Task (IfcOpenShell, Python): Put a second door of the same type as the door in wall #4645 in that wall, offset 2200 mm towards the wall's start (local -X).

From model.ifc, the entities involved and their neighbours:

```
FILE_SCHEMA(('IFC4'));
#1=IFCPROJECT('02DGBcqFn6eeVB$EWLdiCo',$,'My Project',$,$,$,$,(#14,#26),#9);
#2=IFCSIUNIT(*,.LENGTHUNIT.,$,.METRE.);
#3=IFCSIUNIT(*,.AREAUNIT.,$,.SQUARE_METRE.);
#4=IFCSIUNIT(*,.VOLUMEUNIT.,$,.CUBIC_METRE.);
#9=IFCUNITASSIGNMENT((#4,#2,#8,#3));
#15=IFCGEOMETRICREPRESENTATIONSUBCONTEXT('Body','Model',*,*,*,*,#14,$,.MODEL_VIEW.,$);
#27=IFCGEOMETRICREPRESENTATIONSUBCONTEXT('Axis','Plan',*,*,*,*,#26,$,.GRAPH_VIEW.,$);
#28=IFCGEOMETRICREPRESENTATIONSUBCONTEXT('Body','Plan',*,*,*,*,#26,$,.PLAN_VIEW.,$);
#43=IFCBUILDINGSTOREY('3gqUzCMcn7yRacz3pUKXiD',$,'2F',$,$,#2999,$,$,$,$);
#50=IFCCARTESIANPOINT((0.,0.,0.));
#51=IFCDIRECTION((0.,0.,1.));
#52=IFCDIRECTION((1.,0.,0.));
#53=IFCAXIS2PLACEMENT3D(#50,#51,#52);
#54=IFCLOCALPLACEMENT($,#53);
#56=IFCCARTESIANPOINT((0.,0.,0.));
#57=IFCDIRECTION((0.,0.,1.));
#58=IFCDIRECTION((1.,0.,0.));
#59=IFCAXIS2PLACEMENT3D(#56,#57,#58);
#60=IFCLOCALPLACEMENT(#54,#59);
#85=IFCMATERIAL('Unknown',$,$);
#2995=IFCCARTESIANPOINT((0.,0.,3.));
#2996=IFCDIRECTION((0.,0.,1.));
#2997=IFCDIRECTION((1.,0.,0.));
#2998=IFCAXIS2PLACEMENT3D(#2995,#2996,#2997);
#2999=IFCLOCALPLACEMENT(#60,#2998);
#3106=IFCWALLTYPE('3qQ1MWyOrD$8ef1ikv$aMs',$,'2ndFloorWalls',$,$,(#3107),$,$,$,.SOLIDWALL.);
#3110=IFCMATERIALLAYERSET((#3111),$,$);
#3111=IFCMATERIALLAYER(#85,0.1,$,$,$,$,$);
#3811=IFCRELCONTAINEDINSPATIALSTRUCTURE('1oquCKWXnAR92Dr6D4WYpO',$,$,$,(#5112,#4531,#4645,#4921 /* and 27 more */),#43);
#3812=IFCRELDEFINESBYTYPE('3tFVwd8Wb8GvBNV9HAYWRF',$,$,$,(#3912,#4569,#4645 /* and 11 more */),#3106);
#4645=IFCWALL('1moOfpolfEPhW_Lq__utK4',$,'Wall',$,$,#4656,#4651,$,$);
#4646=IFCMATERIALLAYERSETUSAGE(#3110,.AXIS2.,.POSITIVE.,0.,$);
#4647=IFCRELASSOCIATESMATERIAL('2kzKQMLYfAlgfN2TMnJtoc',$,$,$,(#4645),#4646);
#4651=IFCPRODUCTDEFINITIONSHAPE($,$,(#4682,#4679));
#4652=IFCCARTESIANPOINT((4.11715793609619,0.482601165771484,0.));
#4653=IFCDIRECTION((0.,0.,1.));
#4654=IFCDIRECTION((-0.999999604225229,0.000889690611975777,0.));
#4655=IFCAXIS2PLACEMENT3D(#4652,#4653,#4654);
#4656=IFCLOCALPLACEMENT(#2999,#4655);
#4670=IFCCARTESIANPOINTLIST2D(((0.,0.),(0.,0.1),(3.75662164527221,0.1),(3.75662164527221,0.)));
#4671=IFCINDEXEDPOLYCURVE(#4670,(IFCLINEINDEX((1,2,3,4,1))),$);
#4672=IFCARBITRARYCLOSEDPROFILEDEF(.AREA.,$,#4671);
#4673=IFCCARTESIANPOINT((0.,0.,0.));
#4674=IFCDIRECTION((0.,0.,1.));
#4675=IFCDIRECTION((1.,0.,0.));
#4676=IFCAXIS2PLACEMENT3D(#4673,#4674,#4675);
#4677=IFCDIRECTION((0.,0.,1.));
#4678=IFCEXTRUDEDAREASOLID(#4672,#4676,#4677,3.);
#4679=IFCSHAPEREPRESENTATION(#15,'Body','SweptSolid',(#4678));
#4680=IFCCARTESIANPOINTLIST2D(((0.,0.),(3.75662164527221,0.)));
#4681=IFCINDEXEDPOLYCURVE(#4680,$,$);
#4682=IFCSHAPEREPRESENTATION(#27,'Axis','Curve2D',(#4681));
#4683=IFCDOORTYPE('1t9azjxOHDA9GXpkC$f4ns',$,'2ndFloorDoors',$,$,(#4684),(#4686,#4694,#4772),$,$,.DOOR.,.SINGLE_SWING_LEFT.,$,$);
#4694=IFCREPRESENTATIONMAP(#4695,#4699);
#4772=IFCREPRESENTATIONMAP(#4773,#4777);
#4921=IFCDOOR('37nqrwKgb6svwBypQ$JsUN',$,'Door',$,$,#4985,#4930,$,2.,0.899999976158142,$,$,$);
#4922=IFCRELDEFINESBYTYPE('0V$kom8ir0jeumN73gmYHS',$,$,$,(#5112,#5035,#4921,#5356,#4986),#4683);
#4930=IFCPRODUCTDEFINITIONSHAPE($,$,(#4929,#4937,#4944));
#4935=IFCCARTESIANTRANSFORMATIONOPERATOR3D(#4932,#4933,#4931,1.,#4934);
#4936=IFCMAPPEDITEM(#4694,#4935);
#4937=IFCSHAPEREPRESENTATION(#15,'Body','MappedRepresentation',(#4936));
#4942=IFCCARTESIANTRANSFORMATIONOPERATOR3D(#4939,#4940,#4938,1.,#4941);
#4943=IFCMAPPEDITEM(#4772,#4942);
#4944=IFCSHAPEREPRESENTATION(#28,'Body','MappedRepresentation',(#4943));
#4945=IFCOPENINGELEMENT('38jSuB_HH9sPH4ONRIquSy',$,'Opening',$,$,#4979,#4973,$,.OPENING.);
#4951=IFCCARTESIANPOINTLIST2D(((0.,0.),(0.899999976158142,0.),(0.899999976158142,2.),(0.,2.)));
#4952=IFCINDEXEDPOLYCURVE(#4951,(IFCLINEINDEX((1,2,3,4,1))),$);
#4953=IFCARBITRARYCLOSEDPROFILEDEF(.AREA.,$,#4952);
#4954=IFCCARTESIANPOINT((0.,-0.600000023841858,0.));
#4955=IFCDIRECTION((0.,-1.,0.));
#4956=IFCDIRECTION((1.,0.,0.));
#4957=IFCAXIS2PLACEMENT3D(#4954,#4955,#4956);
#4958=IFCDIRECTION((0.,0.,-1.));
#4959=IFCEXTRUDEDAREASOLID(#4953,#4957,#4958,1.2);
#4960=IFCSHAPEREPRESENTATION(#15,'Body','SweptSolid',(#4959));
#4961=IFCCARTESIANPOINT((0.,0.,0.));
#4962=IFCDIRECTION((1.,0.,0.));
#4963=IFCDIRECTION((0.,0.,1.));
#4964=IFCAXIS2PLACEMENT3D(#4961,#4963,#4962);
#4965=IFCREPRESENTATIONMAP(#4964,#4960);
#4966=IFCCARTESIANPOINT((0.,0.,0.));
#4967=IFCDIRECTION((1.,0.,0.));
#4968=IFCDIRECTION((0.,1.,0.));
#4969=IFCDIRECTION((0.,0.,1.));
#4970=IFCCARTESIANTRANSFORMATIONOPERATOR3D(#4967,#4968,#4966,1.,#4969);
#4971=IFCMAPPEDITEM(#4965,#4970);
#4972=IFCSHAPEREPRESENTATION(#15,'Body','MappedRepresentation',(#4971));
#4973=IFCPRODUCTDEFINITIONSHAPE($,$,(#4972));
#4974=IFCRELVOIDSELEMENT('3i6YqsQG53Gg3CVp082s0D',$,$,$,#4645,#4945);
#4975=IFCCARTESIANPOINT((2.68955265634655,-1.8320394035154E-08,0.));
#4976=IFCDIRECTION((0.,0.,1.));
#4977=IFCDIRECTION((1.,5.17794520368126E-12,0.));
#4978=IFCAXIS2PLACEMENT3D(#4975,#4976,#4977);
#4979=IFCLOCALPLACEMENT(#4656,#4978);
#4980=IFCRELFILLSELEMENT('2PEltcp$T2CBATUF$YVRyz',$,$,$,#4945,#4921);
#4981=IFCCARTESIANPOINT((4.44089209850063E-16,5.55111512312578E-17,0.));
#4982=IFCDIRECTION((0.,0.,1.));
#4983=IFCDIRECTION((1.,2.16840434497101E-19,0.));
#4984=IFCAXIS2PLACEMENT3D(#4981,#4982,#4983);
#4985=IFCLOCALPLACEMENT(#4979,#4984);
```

```python
import ifcopenshell
import ifcopenshell.api.feature
import ifcopenshell.api.geometry
import ifcopenshell.api.root
import ifcopenshell.geom
import ifcopenshell.util.element
import ifcopenshell.util.placement
import ifcopenshell.util.shape
import ifcopenshell.util.unit

model = ifcopenshell.open("model.ifc")
unit_scale = ifcopenshell.util.unit.calculate_unit_scale(model)
settings = ifcopenshell.geom.settings()


def volume(element):
    """Net volume in cubic metres, openings subtracted."""
    shape = ifcopenshell.geom.create_shape(settings, element)
    return ifcopenshell.util.shape.get_volume(shape.geometry)


door = model.by_guid("37nqrwKgb6svwBypQ$JsUN")
opening = door.FillsVoids[0].RelatingOpeningElement
wall = opening.VoidsElements[0].RelatingBuildingElement
before = volume(wall)
shift = ifcopenshell.util.placement.get_local_placement(wall.ObjectPlacement)[:3, 0] * -2.2 / unit_scale

# copy_class copies the void relationship, type, container and properties, but no geometry.
new_opening = ifcopenshell.api.root.copy_class(model, product=opening)
new_opening.Representation = ifcopenshell.util.element.copy_deep(
    model, opening.Representation, exclude=["IfcGeometricRepresentationContext", "IfcRepresentationMap"]
)
new_door = ifcopenshell.api.root.copy_class(model, product=door)
new_door.Representation = ifcopenshell.util.element.copy_deep(
    model, door.Representation, exclude=["IfcGeometricRepresentationContext", "IfcRepresentationMap"]
)
ifcopenshell.api.feature.add_filling(model, opening=new_opening, element=new_door)

for old, new in ((opening, new_opening), (door, new_door)):
    matrix = ifcopenshell.util.placement.get_local_placement(old.ObjectPlacement)
    matrix[:3, 3] += shift
    ifcopenshell.api.geometry.edit_object_placement(model, product=new, matrix=matrix, is_si=False)

after = volume(wall)

print(f"wall volume {before:.3f} -> {after:.3f} m3")

model.write("model-out.ifc")
```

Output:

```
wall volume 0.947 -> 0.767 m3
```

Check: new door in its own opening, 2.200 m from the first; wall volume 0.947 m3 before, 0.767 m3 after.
